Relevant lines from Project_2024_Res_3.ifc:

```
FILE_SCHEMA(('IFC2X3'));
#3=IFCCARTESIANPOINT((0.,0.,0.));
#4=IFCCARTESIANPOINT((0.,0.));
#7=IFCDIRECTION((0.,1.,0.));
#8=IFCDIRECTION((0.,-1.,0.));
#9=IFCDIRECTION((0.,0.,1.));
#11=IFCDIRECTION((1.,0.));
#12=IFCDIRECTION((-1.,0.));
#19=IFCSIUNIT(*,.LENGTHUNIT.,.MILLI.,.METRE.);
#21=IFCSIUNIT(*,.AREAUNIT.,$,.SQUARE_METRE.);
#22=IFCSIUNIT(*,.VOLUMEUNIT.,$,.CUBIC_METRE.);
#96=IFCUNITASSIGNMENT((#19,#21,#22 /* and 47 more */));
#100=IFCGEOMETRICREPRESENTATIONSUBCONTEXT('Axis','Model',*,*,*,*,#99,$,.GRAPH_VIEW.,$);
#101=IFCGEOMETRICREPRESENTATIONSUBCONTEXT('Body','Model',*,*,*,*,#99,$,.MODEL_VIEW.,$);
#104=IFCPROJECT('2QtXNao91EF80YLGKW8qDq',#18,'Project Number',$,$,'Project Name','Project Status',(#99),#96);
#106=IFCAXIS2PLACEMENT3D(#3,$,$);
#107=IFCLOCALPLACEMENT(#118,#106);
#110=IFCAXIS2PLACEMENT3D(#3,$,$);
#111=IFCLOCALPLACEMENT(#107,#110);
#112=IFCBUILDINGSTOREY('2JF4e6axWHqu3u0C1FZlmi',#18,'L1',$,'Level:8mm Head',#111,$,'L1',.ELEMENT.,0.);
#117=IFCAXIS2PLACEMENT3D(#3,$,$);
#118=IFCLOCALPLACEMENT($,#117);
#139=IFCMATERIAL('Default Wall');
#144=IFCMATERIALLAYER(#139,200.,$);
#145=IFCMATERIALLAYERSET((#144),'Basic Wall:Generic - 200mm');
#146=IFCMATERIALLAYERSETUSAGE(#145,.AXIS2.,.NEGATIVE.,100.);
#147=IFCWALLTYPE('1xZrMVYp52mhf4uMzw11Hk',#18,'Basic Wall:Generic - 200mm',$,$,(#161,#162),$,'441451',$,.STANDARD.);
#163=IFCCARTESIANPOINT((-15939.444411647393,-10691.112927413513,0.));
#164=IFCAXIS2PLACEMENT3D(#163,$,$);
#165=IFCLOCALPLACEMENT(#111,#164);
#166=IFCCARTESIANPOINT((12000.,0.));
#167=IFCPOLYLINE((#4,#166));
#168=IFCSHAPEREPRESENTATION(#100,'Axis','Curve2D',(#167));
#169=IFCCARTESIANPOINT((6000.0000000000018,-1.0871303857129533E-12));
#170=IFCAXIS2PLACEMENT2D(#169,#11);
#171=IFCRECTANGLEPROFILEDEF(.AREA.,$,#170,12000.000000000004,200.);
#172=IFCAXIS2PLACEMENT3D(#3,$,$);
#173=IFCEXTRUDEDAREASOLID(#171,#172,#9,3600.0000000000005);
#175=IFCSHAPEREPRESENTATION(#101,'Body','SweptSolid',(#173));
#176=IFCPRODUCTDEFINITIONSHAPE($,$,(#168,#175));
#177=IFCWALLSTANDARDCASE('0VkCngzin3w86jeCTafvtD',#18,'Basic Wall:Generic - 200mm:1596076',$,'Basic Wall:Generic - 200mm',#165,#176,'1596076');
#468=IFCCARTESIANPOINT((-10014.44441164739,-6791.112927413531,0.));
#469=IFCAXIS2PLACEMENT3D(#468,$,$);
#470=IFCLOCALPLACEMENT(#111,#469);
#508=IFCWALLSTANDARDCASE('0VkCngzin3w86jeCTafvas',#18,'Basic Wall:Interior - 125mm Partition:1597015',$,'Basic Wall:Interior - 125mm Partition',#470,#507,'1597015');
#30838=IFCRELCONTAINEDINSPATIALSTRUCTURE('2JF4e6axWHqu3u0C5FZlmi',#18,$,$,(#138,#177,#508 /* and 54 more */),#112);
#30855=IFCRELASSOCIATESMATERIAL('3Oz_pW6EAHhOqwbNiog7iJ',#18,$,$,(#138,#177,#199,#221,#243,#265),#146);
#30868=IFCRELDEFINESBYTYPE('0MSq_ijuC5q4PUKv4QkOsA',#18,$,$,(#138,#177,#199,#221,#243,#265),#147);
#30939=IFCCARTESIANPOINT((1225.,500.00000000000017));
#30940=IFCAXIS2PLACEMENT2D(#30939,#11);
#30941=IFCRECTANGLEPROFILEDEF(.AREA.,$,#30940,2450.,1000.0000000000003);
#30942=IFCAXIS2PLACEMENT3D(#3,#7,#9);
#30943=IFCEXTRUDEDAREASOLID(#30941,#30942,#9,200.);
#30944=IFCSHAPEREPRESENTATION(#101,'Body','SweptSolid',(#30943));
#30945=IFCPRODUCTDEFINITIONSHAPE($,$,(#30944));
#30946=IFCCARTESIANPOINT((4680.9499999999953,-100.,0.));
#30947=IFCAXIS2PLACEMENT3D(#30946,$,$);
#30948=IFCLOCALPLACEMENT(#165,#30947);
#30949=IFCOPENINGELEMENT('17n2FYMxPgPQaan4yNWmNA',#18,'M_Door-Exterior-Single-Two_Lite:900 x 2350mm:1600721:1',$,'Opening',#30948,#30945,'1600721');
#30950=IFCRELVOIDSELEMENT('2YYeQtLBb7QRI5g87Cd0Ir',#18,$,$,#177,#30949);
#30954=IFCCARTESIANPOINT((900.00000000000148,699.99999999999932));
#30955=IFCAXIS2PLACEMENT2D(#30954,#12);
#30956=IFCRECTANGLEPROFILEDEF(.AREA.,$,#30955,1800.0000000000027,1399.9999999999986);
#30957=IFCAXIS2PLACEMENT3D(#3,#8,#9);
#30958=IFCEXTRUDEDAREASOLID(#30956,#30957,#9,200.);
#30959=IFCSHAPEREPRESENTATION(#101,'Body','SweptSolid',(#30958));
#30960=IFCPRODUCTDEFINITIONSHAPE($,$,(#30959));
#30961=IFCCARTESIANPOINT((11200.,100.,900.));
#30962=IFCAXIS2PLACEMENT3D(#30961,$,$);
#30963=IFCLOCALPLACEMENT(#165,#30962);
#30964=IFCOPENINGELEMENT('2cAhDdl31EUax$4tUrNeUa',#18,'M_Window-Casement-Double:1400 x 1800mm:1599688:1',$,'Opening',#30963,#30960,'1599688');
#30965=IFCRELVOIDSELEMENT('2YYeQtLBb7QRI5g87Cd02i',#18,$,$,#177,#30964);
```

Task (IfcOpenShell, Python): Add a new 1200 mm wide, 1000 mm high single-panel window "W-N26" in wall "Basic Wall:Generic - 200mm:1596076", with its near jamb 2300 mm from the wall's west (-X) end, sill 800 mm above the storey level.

```python
import numpy as np
import ifcopenshell
import ifcopenshell.api.feature
import ifcopenshell.api.geometry
import ifcopenshell.api.root
import ifcopenshell.api.spatial
import ifcopenshell.api.type
import ifcopenshell.geom
import ifcopenshell.util.element
import ifcopenshell.util.placement
import ifcopenshell.util.representation
import ifcopenshell.util.shape
import ifcopenshell.util.unit

model = ifcopenshell.open("Project_2024_Res_3.ifc")
unit_scale = ifcopenshell.util.unit.calculate_unit_scale(model)
settings = ifcopenshell.geom.settings()


def volume(element):
    """Net volume in cubic metres, openings subtracted."""
    shape = ifcopenshell.geom.create_shape(settings, element)
    return ifcopenshell.util.shape.get_volume(shape.geometry)


wall = model.by_guid("0VkCngzin3w86jeCTafvtD")
storey = ifcopenshell.util.element.get_container(wall, ifc_class="IfcBuildingStorey")
context = ifcopenshell.util.representation.get_context(model, "Model", "Body", "MODEL_VIEW")
before = volume(wall)

width, height, from_end, sill = 1.2, 1, 2.3, 0.8  # metres

# The wall runs along its own X axis, and the end named is its -X end.
wall_shape = ifcopenshell.geom.create_shape(settings, wall)
x, y, z = ifcopenshell.util.shape.get_vertices(wall_shape.geometry).T
start = x.min() + from_end
face, thickness = float(y.min()), float(y.max() - y.min())
wall_matrix = ifcopenshell.util.placement.get_local_placement(wall.ObjectPlacement)
level = ifcopenshell.util.placement.get_local_placement(storey.ObjectPlacement)[2, 3]


def in_wall(x, y):
    """Placement at x, y metres in the wall's axes, at sill height."""
    matrix = wall_matrix.copy()
    matrix[:, 3] = wall_matrix @ np.array([x / unit_scale, y / unit_scale, 0.0, 1.0])
    matrix[2, 3] = level + sill / unit_scale
    return matrix


# Opening: a box that overshoots both wall faces by 50 mm.
opening = ifcopenshell.api.root.create_entity(model, ifc_class="IfcOpeningElement")
box = ifcopenshell.api.geometry.add_wall_representation(
    model, context=context, length=width, height=height, thickness=thickness + 0.1
)
ifcopenshell.api.geometry.assign_representation(model, product=opening, representation=box)
ifcopenshell.api.geometry.edit_object_placement(model, product=opening, matrix=in_wall(start, face - 0.05), is_si=False)
ifcopenshell.api.feature.add_feature(model, feature=opening, element=wall)

window = ifcopenshell.api.root.create_entity(model, ifc_class="IfcWindow", name="W-N26")
window.OverallWidth, window.OverallHeight = width / unit_scale, height / unit_scale
body = ifcopenshell.api.geometry.add_window_representation(
    model,
    context=context,
    overall_width=window.OverallWidth,
    overall_height=window.OverallHeight,
    partition_type="SINGLE_PANEL",
)
ifcopenshell.api.geometry.assign_representation(model, product=window, representation=body)
ifcopenshell.api.spatial.assign_container(model, products=[window], relating_structure=storey)
fills = ifcopenshell.api.feature.add_filling(model, opening=opening, element=window)
fills.OwnerHistory = window.OwnerHistory  # required in IFC2X3

# IFC2X3 keeps the operation on the window style.
style = ifcopenshell.api.root.create_entity(model, ifc_class="IfcWindowStyle", name="W-N26")
style.OperationType, style.ConstructionType = "SINGLE_PANEL", "NOTDEFINED"
style.ParameterTakesPrecedence = style.Sizeable = False
ifcopenshell.api.type.assign_type(model, related_objects=[window], relating_type=style)

# Centre the window in the wall's thickness.
ifcopenshell.api.geometry.edit_object_placement(model, product=window, matrix=in_wall(start, face), is_si=False)
window_shape = ifcopenshell.geom.create_shape(settings, window)
depth = ifcopenshell.util.shape.get_vertices(window_shape.geometry)[:, 1]
offset = face + thickness / 2 - (depth.min() + depth.max()) / 2
ifcopenshell.api.geometry.edit_object_placement(model, product=window, matrix=in_wall(start, offset), is_si=False)

after = volume(wall)

print(f"wall volume {before:.3f} -> {after:.3f} m3")

model.write("Project_2024_Res_3_v2.ifc")
```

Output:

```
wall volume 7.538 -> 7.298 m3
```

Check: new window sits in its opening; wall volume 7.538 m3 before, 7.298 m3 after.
